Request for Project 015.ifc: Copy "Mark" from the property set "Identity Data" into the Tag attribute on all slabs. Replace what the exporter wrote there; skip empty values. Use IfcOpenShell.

First a look at what the model holds.

```python
import ifcopenshell
import ifcopenshell.util.element

model = ifcopenshell.open("Project 015.ifc")
print(model.schema)
slabs = model.by_type("IfcSlab")
print(len(slabs), "slabs")
for e in slabs[:8]:
    source = ifcopenshell.util.element.get_pset(e, "Identity Data", "Mark")
    target = e.Tag
    print(e.id(), repr(source), repr(target), sep=" | ")
```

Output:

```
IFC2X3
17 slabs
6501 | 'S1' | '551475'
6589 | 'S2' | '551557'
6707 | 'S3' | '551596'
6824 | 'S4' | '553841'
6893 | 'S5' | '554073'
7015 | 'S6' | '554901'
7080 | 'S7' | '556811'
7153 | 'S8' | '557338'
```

```python
import ifcopenshell
import ifcopenshell.util.element

model = ifcopenshell.open("Project 015.ifc")

count = 0
for e in model.by_type("IfcSlab"):
    value = ifcopenshell.util.element.get_pset(e, "Identity Data", "Mark")
    current = e.Tag
    if not value or not value.strip() or current == value:
        continue
    e.Tag = value
    count += 1

print(count, "slabs updated")

model.write("Project 015_v2.ifc")
```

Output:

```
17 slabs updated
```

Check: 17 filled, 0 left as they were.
